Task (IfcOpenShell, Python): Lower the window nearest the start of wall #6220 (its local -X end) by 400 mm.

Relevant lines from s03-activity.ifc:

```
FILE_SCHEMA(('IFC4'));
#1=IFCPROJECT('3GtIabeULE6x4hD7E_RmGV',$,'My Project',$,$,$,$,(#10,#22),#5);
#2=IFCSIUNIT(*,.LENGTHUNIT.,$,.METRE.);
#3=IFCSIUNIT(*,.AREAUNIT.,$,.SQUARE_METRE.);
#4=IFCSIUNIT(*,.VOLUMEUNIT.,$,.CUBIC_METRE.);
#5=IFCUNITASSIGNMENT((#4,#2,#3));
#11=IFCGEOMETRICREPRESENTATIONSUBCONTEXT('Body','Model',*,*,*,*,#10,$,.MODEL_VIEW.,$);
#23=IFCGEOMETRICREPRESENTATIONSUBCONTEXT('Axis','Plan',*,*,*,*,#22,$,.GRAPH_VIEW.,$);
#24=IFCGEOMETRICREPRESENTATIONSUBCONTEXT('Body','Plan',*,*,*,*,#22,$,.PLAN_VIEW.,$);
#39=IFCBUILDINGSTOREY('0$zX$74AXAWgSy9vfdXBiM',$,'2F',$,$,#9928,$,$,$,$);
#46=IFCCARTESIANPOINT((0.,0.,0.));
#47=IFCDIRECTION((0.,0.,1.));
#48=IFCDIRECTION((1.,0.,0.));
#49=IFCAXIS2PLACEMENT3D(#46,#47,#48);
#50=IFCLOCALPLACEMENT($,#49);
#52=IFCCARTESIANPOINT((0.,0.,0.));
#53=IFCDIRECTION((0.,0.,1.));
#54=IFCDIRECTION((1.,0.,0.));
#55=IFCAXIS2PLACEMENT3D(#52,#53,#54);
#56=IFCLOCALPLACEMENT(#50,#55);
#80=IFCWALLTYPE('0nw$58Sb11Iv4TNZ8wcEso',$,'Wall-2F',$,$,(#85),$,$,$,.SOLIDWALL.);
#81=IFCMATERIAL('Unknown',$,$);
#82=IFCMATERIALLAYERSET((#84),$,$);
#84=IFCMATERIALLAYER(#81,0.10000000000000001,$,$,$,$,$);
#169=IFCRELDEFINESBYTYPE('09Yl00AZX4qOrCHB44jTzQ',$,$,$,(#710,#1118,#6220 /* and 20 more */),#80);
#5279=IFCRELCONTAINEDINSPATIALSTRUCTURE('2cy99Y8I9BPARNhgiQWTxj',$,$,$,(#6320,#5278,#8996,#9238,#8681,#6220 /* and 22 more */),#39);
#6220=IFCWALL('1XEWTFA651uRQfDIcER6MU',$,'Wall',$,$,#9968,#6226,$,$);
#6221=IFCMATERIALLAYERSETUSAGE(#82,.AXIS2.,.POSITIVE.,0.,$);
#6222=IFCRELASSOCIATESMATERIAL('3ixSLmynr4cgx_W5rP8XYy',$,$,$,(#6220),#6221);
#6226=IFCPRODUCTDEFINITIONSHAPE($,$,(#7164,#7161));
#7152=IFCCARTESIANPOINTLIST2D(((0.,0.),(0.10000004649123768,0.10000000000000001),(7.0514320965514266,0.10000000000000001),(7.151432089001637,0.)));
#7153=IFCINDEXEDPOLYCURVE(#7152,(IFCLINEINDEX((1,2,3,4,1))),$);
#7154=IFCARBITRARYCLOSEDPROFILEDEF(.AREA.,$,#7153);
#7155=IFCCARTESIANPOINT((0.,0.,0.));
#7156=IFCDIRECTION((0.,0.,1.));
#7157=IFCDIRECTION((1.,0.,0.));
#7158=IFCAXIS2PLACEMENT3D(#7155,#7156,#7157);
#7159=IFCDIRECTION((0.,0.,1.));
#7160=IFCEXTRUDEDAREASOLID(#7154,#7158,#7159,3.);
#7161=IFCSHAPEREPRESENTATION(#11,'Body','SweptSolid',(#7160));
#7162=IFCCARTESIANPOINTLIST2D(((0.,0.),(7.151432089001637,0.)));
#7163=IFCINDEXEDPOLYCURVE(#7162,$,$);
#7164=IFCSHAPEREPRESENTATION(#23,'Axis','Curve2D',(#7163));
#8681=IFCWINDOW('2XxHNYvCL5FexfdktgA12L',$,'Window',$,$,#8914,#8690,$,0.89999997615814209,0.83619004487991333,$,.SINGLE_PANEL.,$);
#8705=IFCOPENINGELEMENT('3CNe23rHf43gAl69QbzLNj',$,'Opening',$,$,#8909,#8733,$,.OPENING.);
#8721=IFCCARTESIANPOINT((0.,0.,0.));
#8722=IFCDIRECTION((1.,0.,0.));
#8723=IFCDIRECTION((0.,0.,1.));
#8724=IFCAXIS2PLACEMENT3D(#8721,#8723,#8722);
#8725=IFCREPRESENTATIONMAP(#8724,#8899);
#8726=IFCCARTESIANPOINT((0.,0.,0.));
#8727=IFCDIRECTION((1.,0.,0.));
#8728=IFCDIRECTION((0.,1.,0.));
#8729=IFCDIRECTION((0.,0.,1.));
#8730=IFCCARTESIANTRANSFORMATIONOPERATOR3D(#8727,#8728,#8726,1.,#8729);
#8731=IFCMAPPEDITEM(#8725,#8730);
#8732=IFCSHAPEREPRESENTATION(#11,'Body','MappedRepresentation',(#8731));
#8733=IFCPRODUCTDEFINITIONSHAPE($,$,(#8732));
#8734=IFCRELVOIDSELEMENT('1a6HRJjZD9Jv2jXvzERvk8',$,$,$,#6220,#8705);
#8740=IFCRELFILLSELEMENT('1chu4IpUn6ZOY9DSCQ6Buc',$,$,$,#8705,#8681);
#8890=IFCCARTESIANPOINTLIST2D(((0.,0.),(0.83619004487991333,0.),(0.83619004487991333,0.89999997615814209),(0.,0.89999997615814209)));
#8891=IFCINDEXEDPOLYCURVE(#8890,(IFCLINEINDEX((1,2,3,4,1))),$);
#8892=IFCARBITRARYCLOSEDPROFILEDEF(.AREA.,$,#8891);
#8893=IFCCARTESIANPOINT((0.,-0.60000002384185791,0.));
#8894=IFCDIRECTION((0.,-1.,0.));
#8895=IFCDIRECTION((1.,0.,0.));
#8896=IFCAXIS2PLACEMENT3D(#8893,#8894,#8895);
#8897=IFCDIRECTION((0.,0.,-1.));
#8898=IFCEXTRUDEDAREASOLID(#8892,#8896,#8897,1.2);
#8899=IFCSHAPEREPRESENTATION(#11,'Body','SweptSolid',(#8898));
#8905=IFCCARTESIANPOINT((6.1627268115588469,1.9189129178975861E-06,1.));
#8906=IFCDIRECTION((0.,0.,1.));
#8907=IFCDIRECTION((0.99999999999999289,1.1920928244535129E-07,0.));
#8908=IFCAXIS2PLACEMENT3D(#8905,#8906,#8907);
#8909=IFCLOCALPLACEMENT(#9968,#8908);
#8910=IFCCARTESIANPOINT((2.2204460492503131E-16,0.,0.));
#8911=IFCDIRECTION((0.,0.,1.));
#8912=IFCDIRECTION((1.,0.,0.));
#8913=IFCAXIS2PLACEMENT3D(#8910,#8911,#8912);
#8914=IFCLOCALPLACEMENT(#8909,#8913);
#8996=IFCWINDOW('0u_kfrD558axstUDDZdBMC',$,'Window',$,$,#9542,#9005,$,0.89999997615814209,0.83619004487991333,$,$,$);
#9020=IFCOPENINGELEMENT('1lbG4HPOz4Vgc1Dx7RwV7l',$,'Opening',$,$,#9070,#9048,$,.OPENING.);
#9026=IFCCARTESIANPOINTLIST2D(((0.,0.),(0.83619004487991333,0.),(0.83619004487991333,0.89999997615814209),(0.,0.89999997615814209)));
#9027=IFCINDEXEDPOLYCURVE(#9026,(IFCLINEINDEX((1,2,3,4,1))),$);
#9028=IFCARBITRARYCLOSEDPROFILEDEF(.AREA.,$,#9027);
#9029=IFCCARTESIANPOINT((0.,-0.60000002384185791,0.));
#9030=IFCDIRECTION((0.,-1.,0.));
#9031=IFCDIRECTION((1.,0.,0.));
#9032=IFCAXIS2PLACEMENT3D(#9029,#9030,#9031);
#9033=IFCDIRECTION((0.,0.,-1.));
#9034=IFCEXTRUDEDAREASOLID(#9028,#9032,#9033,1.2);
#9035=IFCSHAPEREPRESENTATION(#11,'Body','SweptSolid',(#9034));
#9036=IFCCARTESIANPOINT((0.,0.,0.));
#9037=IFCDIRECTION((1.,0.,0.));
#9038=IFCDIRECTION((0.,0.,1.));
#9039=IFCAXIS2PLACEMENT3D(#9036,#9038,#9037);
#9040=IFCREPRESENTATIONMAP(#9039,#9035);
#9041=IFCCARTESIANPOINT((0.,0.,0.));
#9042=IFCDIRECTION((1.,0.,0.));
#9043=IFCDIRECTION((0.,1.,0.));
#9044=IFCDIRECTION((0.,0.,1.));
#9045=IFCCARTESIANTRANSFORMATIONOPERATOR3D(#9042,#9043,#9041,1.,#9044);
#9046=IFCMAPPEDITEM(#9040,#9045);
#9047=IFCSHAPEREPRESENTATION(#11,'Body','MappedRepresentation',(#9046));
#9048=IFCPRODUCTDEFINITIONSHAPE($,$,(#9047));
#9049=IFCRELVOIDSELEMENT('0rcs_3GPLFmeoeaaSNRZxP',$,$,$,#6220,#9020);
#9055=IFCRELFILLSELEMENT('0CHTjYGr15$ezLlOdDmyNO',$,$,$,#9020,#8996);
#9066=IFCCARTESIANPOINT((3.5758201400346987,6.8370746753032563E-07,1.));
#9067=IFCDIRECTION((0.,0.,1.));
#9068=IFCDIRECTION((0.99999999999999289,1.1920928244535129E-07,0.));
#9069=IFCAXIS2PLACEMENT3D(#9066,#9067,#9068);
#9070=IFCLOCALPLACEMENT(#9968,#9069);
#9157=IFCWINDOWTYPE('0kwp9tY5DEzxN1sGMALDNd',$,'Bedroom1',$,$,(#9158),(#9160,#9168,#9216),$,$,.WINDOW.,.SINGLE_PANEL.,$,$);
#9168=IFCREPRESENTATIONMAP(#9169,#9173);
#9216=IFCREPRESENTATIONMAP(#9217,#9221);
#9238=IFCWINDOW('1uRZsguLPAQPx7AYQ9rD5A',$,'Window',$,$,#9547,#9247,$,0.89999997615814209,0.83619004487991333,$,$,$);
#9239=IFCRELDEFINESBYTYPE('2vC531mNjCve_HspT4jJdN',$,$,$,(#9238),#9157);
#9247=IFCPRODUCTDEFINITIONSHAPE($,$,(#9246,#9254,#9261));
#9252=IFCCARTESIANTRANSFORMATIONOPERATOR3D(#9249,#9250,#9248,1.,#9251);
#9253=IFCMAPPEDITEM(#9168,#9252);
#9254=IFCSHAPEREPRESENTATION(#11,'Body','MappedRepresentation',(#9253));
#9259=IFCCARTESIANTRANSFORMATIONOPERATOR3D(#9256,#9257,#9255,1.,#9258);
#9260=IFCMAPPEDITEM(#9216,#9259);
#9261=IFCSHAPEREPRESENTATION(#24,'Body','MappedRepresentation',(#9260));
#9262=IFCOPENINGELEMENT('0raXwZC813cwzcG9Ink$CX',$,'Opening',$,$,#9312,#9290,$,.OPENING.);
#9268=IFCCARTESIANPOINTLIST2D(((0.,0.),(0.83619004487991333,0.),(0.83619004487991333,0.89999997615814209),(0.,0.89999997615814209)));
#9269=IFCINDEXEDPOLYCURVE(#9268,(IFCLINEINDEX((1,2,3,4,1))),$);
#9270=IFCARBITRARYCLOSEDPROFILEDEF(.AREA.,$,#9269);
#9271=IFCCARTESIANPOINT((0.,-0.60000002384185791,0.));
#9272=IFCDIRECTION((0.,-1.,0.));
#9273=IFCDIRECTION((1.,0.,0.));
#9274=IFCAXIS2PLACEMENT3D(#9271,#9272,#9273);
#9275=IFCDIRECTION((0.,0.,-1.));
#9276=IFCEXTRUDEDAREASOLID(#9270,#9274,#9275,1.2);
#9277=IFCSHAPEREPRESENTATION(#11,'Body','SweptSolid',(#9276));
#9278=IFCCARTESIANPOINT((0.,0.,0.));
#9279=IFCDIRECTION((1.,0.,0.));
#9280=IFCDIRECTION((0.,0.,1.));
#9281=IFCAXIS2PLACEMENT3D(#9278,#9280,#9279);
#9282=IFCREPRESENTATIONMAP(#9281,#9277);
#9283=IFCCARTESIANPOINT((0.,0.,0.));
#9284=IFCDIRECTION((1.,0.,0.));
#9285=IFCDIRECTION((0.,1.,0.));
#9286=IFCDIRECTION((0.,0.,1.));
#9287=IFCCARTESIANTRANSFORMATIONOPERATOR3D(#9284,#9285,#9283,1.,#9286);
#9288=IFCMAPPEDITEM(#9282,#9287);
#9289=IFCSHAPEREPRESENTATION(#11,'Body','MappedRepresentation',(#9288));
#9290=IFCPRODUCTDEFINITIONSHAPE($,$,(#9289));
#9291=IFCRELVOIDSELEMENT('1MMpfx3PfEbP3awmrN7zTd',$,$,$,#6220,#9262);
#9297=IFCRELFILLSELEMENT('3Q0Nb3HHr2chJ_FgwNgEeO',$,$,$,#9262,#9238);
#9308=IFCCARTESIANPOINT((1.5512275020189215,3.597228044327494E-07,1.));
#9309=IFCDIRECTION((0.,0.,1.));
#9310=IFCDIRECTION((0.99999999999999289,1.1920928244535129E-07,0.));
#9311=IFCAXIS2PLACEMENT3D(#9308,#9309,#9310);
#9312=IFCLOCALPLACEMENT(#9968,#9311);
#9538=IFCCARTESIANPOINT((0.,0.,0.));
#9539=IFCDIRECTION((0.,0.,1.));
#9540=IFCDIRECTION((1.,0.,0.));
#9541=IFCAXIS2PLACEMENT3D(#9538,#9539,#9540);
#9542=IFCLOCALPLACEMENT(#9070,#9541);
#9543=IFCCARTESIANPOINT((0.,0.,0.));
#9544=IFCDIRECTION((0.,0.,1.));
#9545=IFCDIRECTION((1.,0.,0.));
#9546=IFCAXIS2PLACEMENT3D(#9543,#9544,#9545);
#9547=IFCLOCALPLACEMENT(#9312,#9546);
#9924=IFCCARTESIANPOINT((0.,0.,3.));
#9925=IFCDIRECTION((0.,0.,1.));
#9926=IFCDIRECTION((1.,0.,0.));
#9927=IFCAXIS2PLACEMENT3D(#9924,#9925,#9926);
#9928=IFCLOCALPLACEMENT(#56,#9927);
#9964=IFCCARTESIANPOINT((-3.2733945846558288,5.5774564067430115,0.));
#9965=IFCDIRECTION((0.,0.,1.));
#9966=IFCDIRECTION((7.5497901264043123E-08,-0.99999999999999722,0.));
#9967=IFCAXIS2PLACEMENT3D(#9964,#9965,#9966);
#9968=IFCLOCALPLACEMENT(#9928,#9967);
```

```python
import numpy as np
import ifcopenshell
import ifcopenshell.api.geometry
import ifcopenshell.util.placement
import ifcopenshell.util.unit

model = ifcopenshell.open("s03-activity.ifc")
unit_scale = ifcopenshell.util.unit.calculate_unit_scale(model)

window = model.by_guid("1uRZsguLPAQPx7AYQ9rD5A")
opening = window.FillsVoids[0].RelatingOpeningElement
dz = -0.4 / unit_scale

shift = np.array([0.0, 0.0, dz])
# The window is placed relative to its opening, so it follows when the opening moves.
matrix = ifcopenshell.util.placement.get_local_placement(opening.ObjectPlacement)
matrix[:3, 3] += shift
ifcopenshell.api.geometry.edit_object_placement(
    model, product=opening, matrix=matrix, is_si=False, should_transform_children=True
)

print(f"moved by {dz * unit_scale:+.3f} m")

model.write("s03-activity_v2.ifc")
```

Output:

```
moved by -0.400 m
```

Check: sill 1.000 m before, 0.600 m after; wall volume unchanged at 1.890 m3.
